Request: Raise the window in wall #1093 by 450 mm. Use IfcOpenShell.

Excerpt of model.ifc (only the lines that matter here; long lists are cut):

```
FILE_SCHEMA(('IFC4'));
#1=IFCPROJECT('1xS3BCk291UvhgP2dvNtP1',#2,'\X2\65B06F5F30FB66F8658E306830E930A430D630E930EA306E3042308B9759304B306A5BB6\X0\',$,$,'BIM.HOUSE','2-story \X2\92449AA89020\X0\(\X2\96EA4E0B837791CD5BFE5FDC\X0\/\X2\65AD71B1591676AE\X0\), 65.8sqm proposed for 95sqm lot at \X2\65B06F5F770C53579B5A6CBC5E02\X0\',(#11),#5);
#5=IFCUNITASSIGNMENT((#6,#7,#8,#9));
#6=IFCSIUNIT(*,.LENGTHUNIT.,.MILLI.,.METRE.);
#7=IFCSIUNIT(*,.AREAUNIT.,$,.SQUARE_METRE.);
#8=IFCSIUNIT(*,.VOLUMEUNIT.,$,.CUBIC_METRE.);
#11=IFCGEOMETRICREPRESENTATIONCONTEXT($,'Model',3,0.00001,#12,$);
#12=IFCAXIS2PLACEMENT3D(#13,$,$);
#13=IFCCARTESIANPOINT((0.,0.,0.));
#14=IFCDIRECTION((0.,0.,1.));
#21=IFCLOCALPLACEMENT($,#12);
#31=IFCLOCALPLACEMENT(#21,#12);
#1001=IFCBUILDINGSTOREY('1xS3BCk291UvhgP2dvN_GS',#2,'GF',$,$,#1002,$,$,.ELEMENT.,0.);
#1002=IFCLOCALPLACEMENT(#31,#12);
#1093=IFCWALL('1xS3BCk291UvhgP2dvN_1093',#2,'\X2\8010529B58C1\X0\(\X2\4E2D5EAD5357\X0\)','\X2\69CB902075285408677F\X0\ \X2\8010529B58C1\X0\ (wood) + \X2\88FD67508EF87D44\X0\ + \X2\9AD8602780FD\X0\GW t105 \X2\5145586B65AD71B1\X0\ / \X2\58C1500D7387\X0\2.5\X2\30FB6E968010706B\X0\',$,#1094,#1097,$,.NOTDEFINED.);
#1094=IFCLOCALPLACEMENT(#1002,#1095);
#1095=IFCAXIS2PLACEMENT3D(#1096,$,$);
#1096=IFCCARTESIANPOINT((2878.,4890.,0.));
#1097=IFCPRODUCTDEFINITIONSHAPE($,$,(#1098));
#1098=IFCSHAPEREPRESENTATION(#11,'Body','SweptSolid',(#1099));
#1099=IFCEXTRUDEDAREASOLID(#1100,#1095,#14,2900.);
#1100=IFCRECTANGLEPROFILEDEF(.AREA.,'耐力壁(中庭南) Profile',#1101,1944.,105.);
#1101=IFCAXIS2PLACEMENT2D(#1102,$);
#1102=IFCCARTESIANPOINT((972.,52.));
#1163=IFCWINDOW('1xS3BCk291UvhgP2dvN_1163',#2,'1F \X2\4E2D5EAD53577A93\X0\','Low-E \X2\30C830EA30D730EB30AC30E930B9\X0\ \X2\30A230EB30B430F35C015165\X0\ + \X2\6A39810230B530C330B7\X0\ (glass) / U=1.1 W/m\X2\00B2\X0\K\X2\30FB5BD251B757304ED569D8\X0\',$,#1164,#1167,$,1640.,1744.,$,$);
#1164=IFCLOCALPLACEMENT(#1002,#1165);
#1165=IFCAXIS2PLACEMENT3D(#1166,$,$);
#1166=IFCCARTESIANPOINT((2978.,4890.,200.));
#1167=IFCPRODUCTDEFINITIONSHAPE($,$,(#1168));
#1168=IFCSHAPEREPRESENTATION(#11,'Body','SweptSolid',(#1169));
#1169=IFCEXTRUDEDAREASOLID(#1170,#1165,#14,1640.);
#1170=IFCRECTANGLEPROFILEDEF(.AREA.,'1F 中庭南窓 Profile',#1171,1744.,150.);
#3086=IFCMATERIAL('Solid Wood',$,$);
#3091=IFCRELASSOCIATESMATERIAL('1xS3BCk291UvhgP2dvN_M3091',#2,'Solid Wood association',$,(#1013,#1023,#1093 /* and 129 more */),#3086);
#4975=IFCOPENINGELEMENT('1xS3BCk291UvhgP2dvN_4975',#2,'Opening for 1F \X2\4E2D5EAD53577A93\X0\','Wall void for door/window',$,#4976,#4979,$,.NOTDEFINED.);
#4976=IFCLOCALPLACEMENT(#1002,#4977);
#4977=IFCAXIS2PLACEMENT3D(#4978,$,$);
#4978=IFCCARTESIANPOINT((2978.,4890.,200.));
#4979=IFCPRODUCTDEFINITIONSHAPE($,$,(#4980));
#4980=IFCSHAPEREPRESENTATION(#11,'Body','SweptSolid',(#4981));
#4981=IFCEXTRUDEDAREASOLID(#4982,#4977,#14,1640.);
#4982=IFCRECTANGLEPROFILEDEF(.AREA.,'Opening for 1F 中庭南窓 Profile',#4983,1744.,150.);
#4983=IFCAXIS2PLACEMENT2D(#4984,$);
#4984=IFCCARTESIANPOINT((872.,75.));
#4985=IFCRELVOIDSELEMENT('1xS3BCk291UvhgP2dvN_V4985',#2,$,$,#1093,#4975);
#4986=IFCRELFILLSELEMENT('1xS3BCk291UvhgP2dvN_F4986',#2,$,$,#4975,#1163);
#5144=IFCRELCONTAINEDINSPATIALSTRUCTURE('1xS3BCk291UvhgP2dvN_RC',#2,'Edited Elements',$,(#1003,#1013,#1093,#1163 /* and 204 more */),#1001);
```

```python
import numpy as np
import ifcopenshell
import ifcopenshell.api.geometry
import ifcopenshell.util.placement
import ifcopenshell.util.unit

model = ifcopenshell.open("model.ifc")
unit_scale = ifcopenshell.util.unit.calculate_unit_scale(model)

window = model.by_guid("1xS3BCk291UvhgP2dvN_1163")
opening = window.FillsVoids[0].RelatingOpeningElement
dz = 0.45 / unit_scale

shift = np.array([0.0, 0.0, dz])
# The window is not placed relative to its opening, so move both.
for product in (opening, window):
    matrix = ifcopenshell.util.placement.get_local_placement(product.ObjectPlacement)
    matrix[:3, 3] += shift
    ifcopenshell.api.geometry.edit_object_placement(model, product=product, matrix=matrix, is_si=False)

print(f"moved by {dz * unit_scale:+.3f} m")

model.write("model-out.ifc")
```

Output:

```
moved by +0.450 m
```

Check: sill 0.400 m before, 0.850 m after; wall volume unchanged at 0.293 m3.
